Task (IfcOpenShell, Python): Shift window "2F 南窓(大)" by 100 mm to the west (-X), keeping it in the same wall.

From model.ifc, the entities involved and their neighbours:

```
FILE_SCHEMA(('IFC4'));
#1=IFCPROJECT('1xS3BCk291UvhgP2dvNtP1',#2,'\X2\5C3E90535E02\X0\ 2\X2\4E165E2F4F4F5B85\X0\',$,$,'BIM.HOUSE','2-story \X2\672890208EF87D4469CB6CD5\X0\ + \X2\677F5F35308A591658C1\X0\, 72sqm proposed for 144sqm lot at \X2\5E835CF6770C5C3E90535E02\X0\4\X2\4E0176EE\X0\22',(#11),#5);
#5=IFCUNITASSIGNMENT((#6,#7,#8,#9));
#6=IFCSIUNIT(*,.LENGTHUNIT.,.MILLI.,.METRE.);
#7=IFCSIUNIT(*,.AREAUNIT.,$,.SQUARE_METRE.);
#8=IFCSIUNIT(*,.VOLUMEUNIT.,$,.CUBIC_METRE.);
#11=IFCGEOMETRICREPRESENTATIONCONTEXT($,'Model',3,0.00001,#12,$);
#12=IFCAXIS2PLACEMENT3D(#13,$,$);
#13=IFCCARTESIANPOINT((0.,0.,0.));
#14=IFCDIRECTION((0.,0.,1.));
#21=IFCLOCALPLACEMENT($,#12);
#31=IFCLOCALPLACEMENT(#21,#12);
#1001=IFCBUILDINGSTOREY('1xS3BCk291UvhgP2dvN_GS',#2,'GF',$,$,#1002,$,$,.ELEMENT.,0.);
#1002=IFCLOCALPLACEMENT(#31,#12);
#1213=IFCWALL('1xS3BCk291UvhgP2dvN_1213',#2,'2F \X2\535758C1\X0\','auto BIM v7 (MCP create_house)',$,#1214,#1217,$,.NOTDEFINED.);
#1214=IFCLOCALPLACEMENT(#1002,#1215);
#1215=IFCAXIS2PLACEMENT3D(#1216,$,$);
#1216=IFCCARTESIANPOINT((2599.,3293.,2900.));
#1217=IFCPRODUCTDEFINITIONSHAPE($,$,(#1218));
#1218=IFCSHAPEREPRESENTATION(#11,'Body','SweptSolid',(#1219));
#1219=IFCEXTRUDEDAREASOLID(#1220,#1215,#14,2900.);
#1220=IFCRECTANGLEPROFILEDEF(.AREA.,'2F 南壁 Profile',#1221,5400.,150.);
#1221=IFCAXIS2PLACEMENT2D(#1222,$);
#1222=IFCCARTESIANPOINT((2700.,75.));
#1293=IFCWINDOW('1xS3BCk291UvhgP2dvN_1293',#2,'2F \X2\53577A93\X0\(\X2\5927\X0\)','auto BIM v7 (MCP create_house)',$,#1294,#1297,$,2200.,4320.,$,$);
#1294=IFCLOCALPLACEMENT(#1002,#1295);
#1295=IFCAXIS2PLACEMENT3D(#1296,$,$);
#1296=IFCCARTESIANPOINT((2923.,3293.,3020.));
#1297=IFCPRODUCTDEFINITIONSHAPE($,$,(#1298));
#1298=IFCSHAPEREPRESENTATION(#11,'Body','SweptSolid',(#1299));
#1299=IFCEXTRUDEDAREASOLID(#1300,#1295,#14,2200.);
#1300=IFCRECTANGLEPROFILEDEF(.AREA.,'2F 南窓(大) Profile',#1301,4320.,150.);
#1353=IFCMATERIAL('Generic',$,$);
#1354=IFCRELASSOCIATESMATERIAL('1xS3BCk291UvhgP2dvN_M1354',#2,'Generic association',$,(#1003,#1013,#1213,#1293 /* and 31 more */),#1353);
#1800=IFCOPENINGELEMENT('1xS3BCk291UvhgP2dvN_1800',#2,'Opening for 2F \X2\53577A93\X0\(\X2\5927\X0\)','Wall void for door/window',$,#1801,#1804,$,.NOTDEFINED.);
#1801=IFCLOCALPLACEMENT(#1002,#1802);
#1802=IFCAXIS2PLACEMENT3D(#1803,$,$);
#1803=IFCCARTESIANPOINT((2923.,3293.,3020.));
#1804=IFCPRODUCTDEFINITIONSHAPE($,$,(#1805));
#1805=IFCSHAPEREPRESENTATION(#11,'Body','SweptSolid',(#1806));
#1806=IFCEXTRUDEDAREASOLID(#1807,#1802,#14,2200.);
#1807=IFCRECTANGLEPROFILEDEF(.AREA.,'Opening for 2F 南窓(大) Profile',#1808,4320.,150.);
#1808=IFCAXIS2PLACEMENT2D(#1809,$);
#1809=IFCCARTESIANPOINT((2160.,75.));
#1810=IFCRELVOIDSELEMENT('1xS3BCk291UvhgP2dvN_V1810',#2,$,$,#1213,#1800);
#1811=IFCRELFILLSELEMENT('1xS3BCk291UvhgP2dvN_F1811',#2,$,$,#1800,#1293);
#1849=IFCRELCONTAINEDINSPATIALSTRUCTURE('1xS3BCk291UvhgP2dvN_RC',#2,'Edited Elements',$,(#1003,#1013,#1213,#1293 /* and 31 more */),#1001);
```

```python
import ifcopenshell
import ifcopenshell.api.geometry
import ifcopenshell.util.placement
import ifcopenshell.util.unit

model = ifcopenshell.open("model.ifc")
unit_scale = ifcopenshell.util.unit.calculate_unit_scale(model)

window = model.by_guid("1xS3BCk291UvhgP2dvN_1293")
opening = window.FillsVoids[0].RelatingOpeningElement
wall = opening.VoidsElements[0].RelatingBuildingElement

wall_matrix = ifcopenshell.util.placement.get_local_placement(wall.ObjectPlacement)
shift = wall_matrix[:3, 0] * -0.1 / unit_scale
before = ifcopenshell.util.placement.get_local_placement(window.ObjectPlacement)[:3, 3].copy()

# The window is not placed relative to its opening, so move both.
for product in (opening, window):
    matrix = ifcopenshell.util.placement.get_local_placement(product.ObjectPlacement)
    matrix[:3, 3] += shift
    ifcopenshell.api.geometry.edit_object_placement(model, product=product, matrix=matrix, is_si=False)

after = ifcopenshell.util.placement.get_local_placement(window.ObjectPlacement)[:3, 3]
print("window moved by", (after - before).round(3) + 0.0)

model.write("model_v2.ifc")
```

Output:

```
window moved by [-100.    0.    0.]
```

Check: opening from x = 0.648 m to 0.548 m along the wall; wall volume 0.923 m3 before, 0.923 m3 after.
